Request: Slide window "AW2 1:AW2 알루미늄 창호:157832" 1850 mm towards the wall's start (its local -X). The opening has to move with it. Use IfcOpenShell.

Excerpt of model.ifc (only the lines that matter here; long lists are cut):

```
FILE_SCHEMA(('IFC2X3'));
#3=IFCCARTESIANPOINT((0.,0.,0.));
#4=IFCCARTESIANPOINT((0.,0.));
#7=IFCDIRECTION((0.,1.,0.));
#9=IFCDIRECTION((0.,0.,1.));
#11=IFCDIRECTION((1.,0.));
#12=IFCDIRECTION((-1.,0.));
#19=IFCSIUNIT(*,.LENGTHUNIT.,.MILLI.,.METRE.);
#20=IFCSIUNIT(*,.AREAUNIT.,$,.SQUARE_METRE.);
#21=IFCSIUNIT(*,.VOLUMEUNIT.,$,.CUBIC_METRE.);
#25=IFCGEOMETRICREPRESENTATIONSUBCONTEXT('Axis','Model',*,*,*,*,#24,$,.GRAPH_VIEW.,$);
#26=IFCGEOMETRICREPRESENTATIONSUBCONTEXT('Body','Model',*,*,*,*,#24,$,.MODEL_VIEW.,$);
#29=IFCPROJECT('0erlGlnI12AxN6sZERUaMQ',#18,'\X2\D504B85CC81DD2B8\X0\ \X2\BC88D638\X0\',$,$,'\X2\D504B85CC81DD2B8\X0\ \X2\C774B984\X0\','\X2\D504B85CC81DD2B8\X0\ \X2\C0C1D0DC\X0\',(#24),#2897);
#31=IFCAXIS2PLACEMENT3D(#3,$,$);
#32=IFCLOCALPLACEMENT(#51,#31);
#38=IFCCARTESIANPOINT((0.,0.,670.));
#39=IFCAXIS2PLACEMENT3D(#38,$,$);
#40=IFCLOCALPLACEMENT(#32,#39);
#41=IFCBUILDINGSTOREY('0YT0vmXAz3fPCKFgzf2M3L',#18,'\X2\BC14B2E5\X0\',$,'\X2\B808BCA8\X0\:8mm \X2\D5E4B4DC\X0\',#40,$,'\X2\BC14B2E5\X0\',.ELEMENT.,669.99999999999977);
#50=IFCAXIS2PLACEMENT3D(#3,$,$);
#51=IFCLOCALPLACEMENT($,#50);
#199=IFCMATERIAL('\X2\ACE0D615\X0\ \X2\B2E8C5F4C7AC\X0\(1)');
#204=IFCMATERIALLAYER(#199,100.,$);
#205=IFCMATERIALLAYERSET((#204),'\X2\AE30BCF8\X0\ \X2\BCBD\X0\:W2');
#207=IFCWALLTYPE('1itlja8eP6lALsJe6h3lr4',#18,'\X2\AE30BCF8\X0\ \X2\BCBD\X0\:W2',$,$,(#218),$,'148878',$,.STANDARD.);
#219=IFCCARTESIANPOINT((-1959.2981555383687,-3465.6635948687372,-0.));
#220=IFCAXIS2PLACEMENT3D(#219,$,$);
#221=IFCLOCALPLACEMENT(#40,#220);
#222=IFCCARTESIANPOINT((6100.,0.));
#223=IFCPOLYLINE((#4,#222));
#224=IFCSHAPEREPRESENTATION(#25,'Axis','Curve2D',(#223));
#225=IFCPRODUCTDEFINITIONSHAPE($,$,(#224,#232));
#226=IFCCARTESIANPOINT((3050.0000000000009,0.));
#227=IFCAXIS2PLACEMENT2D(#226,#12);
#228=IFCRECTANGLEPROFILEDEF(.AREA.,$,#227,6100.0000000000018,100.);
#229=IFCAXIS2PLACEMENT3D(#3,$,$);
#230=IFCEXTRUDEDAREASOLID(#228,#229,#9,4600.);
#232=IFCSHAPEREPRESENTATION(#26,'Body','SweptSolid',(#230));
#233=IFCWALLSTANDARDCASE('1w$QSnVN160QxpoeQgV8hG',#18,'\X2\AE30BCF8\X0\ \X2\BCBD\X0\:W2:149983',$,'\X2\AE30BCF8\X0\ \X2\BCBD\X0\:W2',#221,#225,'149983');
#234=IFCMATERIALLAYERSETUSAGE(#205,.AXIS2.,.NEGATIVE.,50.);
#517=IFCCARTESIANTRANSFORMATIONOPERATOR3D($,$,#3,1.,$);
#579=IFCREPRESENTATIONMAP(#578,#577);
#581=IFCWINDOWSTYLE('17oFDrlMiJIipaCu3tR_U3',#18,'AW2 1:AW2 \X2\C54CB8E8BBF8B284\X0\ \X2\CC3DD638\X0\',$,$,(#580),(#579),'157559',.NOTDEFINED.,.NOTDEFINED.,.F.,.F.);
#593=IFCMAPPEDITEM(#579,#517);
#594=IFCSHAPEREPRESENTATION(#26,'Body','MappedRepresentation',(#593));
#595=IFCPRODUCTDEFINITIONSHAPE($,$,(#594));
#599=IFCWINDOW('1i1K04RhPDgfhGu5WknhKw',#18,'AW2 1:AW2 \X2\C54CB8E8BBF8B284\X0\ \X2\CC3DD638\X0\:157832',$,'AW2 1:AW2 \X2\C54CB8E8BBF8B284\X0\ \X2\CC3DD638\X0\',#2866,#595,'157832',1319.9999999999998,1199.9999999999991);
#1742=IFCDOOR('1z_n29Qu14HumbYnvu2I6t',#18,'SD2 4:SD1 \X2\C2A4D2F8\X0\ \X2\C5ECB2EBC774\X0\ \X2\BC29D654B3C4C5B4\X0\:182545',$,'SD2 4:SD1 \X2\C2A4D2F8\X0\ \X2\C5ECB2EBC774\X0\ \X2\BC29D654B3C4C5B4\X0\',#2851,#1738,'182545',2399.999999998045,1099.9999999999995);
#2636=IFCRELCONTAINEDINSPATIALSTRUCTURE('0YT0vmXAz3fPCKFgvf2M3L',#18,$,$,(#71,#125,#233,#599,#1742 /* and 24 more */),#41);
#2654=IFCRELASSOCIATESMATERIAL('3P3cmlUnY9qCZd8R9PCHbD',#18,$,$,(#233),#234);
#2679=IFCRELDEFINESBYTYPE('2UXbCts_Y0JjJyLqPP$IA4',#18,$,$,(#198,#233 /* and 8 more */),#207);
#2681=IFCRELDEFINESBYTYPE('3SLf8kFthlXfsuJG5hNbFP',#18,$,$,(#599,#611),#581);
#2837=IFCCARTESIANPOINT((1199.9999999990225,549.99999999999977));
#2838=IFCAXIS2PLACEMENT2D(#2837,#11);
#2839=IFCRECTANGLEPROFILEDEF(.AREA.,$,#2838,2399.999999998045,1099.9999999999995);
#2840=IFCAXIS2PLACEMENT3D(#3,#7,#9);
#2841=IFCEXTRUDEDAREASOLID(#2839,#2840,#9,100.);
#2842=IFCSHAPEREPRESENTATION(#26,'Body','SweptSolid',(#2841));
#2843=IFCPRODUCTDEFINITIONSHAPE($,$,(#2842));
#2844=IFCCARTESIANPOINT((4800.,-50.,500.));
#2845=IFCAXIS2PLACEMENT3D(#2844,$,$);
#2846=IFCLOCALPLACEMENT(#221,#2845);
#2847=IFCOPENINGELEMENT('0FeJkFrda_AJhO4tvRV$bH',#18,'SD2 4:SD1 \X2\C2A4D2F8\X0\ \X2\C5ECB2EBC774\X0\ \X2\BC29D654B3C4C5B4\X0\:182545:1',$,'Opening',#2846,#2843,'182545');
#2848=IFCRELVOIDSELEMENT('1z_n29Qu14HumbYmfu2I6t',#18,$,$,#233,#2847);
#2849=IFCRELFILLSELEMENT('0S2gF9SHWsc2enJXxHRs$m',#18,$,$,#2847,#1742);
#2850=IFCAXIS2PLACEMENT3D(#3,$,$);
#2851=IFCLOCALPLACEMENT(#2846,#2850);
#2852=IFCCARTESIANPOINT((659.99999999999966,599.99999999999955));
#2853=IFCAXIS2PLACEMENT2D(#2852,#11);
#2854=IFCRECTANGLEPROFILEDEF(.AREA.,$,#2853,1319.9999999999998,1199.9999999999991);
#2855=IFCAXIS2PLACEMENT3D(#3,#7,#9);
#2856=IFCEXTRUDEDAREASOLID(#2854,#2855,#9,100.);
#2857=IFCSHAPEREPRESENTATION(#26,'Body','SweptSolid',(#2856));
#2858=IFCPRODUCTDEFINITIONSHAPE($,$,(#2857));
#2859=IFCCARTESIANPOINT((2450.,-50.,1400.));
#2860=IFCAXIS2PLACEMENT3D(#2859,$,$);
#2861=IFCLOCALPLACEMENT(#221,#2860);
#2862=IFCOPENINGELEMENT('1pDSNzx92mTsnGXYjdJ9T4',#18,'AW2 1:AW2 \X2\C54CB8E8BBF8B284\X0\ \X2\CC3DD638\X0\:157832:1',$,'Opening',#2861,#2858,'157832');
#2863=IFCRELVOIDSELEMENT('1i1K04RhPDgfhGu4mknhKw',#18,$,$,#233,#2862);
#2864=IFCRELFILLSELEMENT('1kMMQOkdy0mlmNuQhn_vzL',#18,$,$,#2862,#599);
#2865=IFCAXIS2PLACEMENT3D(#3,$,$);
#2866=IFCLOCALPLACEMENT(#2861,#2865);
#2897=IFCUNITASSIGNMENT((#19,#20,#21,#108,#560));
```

```python
import ifcopenshell
import ifcopenshell.api.geometry
import ifcopenshell.util.placement
import ifcopenshell.util.unit

model = ifcopenshell.open("model.ifc")
unit_scale = ifcopenshell.util.unit.calculate_unit_scale(model)

window = model.by_guid("1i1K04RhPDgfhGu5WknhKw")
opening = window.FillsVoids[0].RelatingOpeningElement
wall = opening.VoidsElements[0].RelatingBuildingElement

wall_matrix = ifcopenshell.util.placement.get_local_placement(wall.ObjectPlacement)
shift = wall_matrix[:3, 0] * -1.85 / unit_scale
before = ifcopenshell.util.placement.get_local_placement(window.ObjectPlacement)[:3, 3].copy()

# The window is placed relative to its opening, so it follows when the opening moves.
matrix = ifcopenshell.util.placement.get_local_placement(opening.ObjectPlacement)
matrix[:3, 3] += shift
ifcopenshell.api.geometry.edit_object_placement(
    model, product=opening, matrix=matrix, is_si=False, should_transform_children=True
)

after = ifcopenshell.util.placement.get_local_placement(window.ObjectPlacement)[:3, 3]
print("window moved by", (after - before).round(3) + 0.0)

model.write("model_rev.ifc")
```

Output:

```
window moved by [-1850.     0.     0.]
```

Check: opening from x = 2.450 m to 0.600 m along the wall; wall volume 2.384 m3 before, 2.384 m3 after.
